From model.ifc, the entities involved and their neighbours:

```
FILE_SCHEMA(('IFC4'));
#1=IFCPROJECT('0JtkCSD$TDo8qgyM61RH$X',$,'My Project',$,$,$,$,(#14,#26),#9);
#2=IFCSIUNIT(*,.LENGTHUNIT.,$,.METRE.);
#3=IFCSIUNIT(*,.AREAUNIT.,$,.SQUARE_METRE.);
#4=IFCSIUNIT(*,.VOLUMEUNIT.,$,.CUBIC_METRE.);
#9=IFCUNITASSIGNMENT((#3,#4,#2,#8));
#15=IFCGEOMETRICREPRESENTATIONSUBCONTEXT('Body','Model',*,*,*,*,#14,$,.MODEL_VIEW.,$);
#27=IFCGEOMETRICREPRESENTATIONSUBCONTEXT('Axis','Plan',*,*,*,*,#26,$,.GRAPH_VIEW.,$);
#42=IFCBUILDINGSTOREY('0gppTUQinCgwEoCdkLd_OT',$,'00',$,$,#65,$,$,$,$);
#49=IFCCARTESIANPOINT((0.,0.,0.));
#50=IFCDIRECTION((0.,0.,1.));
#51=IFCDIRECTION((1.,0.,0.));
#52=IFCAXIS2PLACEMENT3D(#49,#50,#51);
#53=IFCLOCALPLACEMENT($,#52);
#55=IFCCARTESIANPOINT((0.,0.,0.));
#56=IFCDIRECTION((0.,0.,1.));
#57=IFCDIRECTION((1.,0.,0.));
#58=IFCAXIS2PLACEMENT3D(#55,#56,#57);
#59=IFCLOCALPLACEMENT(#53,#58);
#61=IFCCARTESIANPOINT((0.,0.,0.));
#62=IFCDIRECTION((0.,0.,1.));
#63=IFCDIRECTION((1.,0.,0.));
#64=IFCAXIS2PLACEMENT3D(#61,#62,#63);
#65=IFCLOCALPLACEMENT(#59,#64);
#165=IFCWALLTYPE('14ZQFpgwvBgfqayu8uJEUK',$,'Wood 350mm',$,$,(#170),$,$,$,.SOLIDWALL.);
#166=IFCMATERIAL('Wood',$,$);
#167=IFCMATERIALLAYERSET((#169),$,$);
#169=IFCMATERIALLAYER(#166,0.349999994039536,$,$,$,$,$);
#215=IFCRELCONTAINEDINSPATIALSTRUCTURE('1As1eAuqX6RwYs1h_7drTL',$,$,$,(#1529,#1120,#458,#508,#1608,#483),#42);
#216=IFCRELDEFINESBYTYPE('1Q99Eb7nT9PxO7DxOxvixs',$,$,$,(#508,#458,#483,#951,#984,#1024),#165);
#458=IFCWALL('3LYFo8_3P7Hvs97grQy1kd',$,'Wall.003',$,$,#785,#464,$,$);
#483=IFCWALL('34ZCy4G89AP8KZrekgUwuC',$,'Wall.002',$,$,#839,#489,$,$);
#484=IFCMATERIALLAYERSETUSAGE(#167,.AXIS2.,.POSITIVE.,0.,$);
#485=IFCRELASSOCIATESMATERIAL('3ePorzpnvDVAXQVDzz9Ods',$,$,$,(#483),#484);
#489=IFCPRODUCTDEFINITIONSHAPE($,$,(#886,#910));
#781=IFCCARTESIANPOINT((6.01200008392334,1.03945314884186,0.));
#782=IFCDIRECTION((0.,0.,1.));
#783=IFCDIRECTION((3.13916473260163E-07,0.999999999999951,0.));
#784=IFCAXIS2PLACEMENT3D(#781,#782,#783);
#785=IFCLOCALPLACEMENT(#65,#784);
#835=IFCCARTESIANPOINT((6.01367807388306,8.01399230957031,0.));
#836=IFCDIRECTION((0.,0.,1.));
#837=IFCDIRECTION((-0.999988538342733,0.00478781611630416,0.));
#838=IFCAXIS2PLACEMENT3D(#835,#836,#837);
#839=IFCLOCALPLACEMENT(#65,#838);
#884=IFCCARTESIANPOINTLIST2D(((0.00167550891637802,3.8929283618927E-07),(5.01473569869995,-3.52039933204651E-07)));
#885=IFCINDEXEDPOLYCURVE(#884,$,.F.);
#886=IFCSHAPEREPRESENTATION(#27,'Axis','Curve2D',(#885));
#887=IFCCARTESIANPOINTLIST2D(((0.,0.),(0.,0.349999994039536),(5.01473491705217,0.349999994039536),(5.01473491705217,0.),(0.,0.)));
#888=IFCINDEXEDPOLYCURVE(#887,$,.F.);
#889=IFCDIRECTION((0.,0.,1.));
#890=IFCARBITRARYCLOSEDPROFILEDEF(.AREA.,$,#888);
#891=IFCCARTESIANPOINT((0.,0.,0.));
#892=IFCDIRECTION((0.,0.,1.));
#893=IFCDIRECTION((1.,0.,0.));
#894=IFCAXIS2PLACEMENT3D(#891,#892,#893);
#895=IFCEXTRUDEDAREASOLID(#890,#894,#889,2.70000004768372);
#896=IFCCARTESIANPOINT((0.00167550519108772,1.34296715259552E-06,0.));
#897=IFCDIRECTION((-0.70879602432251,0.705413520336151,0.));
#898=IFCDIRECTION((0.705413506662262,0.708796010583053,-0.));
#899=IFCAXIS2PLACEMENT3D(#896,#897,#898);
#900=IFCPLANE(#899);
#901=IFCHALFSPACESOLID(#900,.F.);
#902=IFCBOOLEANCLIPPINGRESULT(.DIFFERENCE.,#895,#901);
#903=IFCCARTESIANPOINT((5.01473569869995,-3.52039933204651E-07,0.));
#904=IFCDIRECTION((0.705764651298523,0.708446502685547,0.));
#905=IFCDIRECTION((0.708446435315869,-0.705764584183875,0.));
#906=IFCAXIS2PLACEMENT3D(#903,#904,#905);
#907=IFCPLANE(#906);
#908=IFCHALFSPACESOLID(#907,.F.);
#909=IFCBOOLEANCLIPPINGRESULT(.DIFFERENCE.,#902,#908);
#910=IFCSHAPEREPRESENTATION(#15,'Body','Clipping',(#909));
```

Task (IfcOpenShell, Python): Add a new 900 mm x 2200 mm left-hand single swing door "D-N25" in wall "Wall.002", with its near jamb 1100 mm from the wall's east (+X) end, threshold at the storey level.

```python
import numpy as np
import ifcopenshell
import ifcopenshell.api.feature
import ifcopenshell.api.geometry
import ifcopenshell.api.root
import ifcopenshell.api.spatial
import ifcopenshell.geom
import ifcopenshell.util.element
import ifcopenshell.util.placement
import ifcopenshell.util.representation
import ifcopenshell.util.shape
import ifcopenshell.util.unit

model = ifcopenshell.open("model.ifc")
unit_scale = ifcopenshell.util.unit.calculate_unit_scale(model)
settings = ifcopenshell.geom.settings()


def volume(element):
    """Net volume in cubic metres, openings subtracted."""
    shape = ifcopenshell.geom.create_shape(settings, element)
    return ifcopenshell.util.shape.get_volume(shape.geometry)


wall = model.by_guid("34ZCy4G89AP8KZrekgUwuC")
storey = ifcopenshell.util.element.get_container(wall, ifc_class="IfcBuildingStorey")
context = ifcopenshell.util.representation.get_context(model, "Model", "Body", "MODEL_VIEW")
before = volume(wall)

width, height, from_end, sill = 0.9, 2.2, 1.1, 0.0  # metres

# The wall runs along its own X axis, and the end named is its -X end.
wall_shape = ifcopenshell.geom.create_shape(settings, wall)
x, y, z = ifcopenshell.util.shape.get_vertices(wall_shape.geometry).T
start = x.min() + from_end
face, thickness = float(y.min()), float(y.max() - y.min())
wall_matrix = ifcopenshell.util.placement.get_local_placement(wall.ObjectPlacement)
level = ifcopenshell.util.placement.get_local_placement(storey.ObjectPlacement)[2, 3]


def in_wall(x, y):
    """Placement at x, y metres in the wall's axes, at sill height."""
    matrix = wall_matrix.copy()
    matrix[:, 3] = wall_matrix @ np.array([x / unit_scale, y / unit_scale, 0.0, 1.0])
    matrix[2, 3] = level + sill / unit_scale
    return matrix


# Opening: a box that overshoots both wall faces by 50 mm.
opening = ifcopenshell.api.root.create_entity(model, ifc_class="IfcOpeningElement", predefined_type="OPENING")
box = ifcopenshell.api.geometry.add_wall_representation(
    model, context=context, length=width, height=height, thickness=thickness + 0.1
)
ifcopenshell.api.geometry.assign_representation(model, product=opening, representation=box)
ifcopenshell.api.geometry.edit_object_placement(model, product=opening, matrix=in_wall(start, face - 0.05), is_si=False)
ifcopenshell.api.feature.add_feature(model, feature=opening, element=wall)

door = ifcopenshell.api.root.create_entity(model, ifc_class="IfcDoor", name="D-N25", predefined_type="DOOR")
door.OverallWidth, door.OverallHeight = width / unit_scale, height / unit_scale
door.OperationType = "SINGLE_SWING_LEFT"
body = ifcopenshell.api.geometry.add_door_representation(
    model,
    context=context,
    overall_width=door.OverallWidth,
    overall_height=door.OverallHeight,
    operation_type="SINGLE_SWING_LEFT",
    lining_properties={"LiningDepth": thickness / unit_scale, "ThresholdDepth": thickness / unit_scale},
)
ifcopenshell.api.geometry.assign_representation(model, product=door, representation=body)
ifcopenshell.api.spatial.assign_container(model, products=[door], relating_structure=storey)
ifcopenshell.api.feature.add_filling(model, opening=opening, element=door)

# The lining spans the wall, so the door starts at the wall face.
ifcopenshell.api.geometry.edit_object_placement(model, product=door, matrix=in_wall(start, face), is_si=False)

after = volume(wall)

print(f"wall volume {before:.3f} -> {after:.3f} m3")

model.write("model_edited.ifc")
```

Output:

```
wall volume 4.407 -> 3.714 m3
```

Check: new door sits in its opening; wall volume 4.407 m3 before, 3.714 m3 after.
